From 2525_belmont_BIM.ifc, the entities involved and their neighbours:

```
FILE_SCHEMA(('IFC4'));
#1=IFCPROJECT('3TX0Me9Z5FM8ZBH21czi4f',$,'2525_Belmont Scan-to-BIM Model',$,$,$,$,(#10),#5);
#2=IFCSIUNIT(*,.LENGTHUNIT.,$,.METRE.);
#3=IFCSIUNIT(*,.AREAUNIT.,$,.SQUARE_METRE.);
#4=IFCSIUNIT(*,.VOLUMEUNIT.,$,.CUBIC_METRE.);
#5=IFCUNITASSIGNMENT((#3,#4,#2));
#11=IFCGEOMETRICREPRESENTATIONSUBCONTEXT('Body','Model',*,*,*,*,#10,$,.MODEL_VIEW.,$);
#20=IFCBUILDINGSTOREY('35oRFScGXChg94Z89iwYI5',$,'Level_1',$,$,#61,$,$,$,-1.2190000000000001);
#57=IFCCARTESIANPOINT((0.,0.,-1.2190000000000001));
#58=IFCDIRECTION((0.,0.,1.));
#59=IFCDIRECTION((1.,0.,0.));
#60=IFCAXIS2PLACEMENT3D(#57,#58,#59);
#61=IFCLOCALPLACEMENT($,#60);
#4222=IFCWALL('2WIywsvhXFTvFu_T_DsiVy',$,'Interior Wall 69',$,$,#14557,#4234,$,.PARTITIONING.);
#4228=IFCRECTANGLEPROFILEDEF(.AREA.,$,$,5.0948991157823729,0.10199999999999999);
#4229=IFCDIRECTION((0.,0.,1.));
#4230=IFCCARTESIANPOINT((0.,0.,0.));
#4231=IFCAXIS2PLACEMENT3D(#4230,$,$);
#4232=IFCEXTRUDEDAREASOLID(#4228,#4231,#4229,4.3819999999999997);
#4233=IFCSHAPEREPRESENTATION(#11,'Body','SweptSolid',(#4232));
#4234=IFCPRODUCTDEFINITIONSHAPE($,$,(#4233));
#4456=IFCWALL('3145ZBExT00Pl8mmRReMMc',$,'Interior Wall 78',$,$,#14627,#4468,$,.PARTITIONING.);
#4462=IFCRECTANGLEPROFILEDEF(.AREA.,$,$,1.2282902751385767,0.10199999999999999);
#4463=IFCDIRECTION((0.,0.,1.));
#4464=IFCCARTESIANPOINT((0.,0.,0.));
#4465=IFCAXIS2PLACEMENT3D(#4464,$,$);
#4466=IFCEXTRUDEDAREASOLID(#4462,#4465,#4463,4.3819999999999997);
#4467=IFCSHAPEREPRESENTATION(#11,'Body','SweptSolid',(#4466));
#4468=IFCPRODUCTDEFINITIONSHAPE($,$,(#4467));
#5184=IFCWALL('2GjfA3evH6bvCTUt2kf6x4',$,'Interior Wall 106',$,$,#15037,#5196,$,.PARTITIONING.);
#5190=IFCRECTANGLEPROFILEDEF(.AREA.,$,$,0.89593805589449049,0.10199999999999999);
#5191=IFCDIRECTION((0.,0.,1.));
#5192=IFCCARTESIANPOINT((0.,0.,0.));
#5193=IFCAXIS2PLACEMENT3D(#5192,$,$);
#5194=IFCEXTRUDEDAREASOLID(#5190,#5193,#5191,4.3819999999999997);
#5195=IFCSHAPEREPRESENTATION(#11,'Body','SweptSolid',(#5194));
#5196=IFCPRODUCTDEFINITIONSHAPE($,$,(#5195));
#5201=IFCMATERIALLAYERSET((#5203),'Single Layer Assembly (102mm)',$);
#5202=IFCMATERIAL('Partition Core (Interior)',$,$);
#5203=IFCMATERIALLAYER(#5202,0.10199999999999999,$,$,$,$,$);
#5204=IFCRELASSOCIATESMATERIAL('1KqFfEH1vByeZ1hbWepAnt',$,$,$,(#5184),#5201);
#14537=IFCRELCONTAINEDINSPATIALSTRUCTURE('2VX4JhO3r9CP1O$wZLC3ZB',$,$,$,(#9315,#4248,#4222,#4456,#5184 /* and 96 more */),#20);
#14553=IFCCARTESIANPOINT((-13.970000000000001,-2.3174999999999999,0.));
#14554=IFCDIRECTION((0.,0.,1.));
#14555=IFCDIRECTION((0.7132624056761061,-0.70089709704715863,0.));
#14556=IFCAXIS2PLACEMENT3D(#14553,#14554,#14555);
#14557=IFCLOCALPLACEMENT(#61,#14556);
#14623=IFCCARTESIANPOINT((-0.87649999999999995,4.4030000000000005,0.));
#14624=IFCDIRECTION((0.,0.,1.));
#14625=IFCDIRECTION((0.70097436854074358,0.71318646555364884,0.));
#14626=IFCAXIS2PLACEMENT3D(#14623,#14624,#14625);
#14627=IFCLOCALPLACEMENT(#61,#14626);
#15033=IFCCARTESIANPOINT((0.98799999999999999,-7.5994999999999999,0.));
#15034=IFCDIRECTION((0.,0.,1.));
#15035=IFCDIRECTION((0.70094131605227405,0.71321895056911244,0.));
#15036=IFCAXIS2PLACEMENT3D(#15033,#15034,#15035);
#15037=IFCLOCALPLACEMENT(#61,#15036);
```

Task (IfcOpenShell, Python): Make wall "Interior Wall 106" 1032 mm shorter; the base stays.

```python
import ifcopenshell
import ifcopenshell.geom
import ifcopenshell.util.representation
import ifcopenshell.util.shape

model = ifcopenshell.open("2525_belmont_BIM.ifc")
settings = ifcopenshell.geom.settings()


def volume(element):
    """Net volume in cubic metres, openings subtracted."""
    shape = ifcopenshell.geom.create_shape(settings, element)
    return ifcopenshell.util.shape.get_volume(shape.geometry)


wall = model.by_guid("2GjfA3evH6bvCTUt2kf6x4")
before = volume(wall)

body = ifcopenshell.util.representation.get_representation(wall, "Model", "Body")
solid = body.Items[0]
old_height = solid.Depth
solid.Depth -= 1.032
after = volume(wall)

print(f"height {old_height:g} -> {solid.Depth:g}, volume {before:.3f} -> {after:.3f} m3")

model.write("2525_belmont_BIM-out.ifc")
```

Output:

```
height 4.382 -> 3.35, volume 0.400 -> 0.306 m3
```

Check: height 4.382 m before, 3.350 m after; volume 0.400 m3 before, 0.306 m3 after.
